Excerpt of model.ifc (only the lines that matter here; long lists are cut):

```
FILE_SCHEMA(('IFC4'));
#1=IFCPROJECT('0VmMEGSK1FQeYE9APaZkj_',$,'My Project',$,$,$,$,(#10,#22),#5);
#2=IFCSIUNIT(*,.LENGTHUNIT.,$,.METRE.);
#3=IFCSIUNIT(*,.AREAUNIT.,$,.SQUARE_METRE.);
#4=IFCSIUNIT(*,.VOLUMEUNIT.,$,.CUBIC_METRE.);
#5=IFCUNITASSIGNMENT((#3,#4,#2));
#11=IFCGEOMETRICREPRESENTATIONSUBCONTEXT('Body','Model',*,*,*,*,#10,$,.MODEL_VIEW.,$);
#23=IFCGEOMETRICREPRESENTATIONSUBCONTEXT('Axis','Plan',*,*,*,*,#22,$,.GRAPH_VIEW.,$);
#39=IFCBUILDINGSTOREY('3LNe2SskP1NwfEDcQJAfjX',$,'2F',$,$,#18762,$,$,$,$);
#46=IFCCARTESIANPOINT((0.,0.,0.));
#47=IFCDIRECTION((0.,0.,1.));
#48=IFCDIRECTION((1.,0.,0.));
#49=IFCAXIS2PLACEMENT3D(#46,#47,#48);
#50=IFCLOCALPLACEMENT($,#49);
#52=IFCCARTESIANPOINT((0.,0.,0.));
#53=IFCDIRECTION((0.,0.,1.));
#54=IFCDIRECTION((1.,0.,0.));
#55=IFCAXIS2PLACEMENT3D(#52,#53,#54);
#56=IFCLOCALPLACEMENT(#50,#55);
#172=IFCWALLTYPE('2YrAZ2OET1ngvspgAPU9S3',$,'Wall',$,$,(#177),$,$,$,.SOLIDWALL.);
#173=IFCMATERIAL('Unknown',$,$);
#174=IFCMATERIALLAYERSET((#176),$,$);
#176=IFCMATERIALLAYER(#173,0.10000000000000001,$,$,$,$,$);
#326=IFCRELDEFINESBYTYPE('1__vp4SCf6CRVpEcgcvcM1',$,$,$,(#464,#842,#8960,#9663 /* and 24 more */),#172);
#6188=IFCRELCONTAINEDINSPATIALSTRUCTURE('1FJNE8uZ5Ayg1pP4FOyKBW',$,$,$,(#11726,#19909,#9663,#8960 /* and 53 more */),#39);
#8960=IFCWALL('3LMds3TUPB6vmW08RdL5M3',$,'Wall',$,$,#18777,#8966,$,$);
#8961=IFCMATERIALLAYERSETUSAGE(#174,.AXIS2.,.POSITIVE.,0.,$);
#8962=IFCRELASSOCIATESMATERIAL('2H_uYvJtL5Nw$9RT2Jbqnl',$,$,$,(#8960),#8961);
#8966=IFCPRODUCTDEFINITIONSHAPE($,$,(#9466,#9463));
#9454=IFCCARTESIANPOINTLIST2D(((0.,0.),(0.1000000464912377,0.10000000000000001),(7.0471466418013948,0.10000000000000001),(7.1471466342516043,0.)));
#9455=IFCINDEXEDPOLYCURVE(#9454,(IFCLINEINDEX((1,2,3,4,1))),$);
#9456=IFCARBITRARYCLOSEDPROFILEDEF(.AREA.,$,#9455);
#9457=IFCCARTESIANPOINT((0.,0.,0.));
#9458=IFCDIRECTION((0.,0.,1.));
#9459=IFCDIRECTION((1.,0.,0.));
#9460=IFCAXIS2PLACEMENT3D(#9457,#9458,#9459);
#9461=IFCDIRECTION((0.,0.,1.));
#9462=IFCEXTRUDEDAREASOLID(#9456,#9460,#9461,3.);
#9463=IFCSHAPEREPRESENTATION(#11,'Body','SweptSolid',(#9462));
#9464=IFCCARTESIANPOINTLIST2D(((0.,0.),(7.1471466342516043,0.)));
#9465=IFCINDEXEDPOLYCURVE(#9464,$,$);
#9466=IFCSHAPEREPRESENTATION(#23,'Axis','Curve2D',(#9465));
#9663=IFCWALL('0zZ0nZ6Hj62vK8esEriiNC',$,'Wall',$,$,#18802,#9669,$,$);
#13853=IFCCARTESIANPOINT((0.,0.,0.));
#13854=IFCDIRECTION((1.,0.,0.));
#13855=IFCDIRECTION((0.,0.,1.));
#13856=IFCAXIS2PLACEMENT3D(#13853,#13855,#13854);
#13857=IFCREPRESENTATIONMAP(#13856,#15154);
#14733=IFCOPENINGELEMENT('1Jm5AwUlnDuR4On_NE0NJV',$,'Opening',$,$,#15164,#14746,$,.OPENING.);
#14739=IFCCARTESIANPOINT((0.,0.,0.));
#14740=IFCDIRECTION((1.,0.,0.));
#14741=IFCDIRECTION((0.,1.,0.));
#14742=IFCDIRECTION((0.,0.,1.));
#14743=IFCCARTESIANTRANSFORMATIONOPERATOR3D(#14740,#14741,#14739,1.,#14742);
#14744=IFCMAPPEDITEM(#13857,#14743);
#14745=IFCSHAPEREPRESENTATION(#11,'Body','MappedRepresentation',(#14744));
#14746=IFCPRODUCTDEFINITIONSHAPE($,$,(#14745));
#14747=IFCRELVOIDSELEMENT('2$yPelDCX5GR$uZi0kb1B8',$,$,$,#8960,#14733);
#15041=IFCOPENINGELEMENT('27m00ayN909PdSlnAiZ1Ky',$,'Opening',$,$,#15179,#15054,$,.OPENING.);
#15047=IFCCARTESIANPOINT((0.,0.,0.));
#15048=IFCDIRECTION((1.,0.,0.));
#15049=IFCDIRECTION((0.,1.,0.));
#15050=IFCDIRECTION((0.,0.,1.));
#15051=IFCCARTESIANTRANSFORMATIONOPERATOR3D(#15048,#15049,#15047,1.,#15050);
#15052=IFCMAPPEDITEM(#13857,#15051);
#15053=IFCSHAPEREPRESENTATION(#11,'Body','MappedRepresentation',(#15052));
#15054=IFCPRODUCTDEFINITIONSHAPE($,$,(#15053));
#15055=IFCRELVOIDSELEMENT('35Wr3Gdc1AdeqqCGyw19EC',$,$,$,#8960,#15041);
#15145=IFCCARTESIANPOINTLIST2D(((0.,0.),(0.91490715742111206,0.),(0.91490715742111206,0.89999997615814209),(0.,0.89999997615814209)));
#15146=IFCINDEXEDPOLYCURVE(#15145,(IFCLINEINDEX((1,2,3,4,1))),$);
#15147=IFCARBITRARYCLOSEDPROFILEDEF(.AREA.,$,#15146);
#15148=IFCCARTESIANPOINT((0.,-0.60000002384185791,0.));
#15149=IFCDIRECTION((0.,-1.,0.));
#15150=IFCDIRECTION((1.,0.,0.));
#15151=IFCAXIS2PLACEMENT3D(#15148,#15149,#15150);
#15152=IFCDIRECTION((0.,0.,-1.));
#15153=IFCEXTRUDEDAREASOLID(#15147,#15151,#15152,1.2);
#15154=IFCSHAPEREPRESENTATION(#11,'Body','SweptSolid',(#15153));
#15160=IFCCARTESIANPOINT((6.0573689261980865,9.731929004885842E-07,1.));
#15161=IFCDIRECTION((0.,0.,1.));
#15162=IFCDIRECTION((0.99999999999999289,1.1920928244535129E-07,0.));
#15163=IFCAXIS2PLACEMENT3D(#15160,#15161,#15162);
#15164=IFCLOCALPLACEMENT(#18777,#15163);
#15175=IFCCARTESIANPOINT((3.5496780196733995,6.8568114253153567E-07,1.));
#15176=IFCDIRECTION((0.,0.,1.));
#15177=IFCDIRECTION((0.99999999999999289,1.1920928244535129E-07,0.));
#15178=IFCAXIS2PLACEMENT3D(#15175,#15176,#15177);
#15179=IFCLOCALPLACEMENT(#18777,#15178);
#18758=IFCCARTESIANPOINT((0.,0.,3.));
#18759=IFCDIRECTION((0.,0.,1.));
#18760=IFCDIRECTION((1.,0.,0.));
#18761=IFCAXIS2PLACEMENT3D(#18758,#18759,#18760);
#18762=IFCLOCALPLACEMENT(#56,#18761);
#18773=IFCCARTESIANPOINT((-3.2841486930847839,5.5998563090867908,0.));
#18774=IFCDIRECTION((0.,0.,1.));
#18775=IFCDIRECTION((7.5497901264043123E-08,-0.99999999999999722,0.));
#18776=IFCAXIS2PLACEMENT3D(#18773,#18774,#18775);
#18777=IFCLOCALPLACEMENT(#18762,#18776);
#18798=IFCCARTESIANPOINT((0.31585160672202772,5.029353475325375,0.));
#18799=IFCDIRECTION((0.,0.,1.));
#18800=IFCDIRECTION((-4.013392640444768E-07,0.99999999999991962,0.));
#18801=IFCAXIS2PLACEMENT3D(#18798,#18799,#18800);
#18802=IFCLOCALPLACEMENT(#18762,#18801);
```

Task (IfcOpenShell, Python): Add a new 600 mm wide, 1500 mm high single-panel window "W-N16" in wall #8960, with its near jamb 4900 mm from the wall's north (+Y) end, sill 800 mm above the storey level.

```python
import numpy as np
import ifcopenshell
import ifcopenshell.api.feature
import ifcopenshell.api.geometry
import ifcopenshell.api.root
import ifcopenshell.api.spatial
import ifcopenshell.geom
import ifcopenshell.util.element
import ifcopenshell.util.placement
import ifcopenshell.util.representation
import ifcopenshell.util.shape
import ifcopenshell.util.unit

model = ifcopenshell.open("model.ifc")
unit_scale = ifcopenshell.util.unit.calculate_unit_scale(model)
settings = ifcopenshell.geom.settings()


def volume(element):
    """Net volume in cubic metres, openings subtracted."""
    shape = ifcopenshell.geom.create_shape(settings, element)
    return ifcopenshell.util.shape.get_volume(shape.geometry)


wall = model.by_id(8960)
storey = ifcopenshell.util.element.get_container(wall, ifc_class="IfcBuildingStorey")
context = ifcopenshell.util.representation.get_context(model, "Model", "Body", "MODEL_VIEW")
before = volume(wall)

width, height, from_end, sill = 0.6, 1.5, 4.9, 0.8  # metres

# The wall runs along its own X axis, and the end named is its -X end.
wall_shape = ifcopenshell.geom.create_shape(settings, wall)
x, y, z = ifcopenshell.util.shape.get_vertices(wall_shape.geometry).T
start = x.min() + from_end
face, thickness = float(y.min()), float(y.max() - y.min())
wall_matrix = ifcopenshell.util.placement.get_local_placement(wall.ObjectPlacement)
level = ifcopenshell.util.placement.get_local_placement(storey.ObjectPlacement)[2, 3]


def in_wall(x, y):
    """Placement at x, y metres in the wall's axes, at sill height."""
    matrix = wall_matrix.copy()
    matrix[:, 3] = wall_matrix @ np.array([x / unit_scale, y / unit_scale, 0.0, 1.0])
    matrix[2, 3] = level + sill / unit_scale
    return matrix


# Opening: a box that overshoots both wall faces by 50 mm.
opening = ifcopenshell.api.root.create_entity(model, ifc_class="IfcOpeningElement", predefined_type="OPENING")
box = ifcopenshell.api.geometry.add_wall_representation(
    model, context=context, length=width, height=height, thickness=thickness + 0.1
)
ifcopenshell.api.geometry.assign_representation(model, product=opening, representation=box)
ifcopenshell.api.geometry.edit_object_placement(model, product=opening, matrix=in_wall(start, face - 0.05), is_si=False)
ifcopenshell.api.feature.add_feature(model, feature=opening, element=wall)

window = ifcopenshell.api.root.create_entity(model, ifc_class="IfcWindow", name="W-N16", predefined_type="WINDOW")
window.OverallWidth, window.OverallHeight = width / unit_scale, height / unit_scale
window.PartitioningType = "SINGLE_PANEL"
body = ifcopenshell.api.geometry.add_window_representation(
    model,
    context=context,
    overall_width=window.OverallWidth,
    overall_height=window.OverallHeight,
    partition_type="SINGLE_PANEL",
)
ifcopenshell.api.geometry.assign_representation(model, product=window, representation=body)
ifcopenshell.api.spatial.assign_container(model, products=[window], relating_structure=storey)
ifcopenshell.api.feature.add_filling(model, opening=opening, element=window)

# Centre the window in the wall's thickness.
ifcopenshell.api.geometry.edit_object_placement(model, product=window, matrix=in_wall(start, face), is_si=False)
window_shape = ifcopenshell.geom.create_shape(settings, window)
depth = ifcopenshell.util.shape.get_vertices(window_shape.geometry)[:, 1]
offset = face + thickness / 2 - (depth.min() + depth.max()) / 2
ifcopenshell.api.geometry.edit_object_placement(model, product=window, matrix=in_wall(start, offset), is_si=False)

after = volume(wall)

print(f"wall volume {before:.3f} -> {after:.3f} m3")

model.write("model-out.ifc")
```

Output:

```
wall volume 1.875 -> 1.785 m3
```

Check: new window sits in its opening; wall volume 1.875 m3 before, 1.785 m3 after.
